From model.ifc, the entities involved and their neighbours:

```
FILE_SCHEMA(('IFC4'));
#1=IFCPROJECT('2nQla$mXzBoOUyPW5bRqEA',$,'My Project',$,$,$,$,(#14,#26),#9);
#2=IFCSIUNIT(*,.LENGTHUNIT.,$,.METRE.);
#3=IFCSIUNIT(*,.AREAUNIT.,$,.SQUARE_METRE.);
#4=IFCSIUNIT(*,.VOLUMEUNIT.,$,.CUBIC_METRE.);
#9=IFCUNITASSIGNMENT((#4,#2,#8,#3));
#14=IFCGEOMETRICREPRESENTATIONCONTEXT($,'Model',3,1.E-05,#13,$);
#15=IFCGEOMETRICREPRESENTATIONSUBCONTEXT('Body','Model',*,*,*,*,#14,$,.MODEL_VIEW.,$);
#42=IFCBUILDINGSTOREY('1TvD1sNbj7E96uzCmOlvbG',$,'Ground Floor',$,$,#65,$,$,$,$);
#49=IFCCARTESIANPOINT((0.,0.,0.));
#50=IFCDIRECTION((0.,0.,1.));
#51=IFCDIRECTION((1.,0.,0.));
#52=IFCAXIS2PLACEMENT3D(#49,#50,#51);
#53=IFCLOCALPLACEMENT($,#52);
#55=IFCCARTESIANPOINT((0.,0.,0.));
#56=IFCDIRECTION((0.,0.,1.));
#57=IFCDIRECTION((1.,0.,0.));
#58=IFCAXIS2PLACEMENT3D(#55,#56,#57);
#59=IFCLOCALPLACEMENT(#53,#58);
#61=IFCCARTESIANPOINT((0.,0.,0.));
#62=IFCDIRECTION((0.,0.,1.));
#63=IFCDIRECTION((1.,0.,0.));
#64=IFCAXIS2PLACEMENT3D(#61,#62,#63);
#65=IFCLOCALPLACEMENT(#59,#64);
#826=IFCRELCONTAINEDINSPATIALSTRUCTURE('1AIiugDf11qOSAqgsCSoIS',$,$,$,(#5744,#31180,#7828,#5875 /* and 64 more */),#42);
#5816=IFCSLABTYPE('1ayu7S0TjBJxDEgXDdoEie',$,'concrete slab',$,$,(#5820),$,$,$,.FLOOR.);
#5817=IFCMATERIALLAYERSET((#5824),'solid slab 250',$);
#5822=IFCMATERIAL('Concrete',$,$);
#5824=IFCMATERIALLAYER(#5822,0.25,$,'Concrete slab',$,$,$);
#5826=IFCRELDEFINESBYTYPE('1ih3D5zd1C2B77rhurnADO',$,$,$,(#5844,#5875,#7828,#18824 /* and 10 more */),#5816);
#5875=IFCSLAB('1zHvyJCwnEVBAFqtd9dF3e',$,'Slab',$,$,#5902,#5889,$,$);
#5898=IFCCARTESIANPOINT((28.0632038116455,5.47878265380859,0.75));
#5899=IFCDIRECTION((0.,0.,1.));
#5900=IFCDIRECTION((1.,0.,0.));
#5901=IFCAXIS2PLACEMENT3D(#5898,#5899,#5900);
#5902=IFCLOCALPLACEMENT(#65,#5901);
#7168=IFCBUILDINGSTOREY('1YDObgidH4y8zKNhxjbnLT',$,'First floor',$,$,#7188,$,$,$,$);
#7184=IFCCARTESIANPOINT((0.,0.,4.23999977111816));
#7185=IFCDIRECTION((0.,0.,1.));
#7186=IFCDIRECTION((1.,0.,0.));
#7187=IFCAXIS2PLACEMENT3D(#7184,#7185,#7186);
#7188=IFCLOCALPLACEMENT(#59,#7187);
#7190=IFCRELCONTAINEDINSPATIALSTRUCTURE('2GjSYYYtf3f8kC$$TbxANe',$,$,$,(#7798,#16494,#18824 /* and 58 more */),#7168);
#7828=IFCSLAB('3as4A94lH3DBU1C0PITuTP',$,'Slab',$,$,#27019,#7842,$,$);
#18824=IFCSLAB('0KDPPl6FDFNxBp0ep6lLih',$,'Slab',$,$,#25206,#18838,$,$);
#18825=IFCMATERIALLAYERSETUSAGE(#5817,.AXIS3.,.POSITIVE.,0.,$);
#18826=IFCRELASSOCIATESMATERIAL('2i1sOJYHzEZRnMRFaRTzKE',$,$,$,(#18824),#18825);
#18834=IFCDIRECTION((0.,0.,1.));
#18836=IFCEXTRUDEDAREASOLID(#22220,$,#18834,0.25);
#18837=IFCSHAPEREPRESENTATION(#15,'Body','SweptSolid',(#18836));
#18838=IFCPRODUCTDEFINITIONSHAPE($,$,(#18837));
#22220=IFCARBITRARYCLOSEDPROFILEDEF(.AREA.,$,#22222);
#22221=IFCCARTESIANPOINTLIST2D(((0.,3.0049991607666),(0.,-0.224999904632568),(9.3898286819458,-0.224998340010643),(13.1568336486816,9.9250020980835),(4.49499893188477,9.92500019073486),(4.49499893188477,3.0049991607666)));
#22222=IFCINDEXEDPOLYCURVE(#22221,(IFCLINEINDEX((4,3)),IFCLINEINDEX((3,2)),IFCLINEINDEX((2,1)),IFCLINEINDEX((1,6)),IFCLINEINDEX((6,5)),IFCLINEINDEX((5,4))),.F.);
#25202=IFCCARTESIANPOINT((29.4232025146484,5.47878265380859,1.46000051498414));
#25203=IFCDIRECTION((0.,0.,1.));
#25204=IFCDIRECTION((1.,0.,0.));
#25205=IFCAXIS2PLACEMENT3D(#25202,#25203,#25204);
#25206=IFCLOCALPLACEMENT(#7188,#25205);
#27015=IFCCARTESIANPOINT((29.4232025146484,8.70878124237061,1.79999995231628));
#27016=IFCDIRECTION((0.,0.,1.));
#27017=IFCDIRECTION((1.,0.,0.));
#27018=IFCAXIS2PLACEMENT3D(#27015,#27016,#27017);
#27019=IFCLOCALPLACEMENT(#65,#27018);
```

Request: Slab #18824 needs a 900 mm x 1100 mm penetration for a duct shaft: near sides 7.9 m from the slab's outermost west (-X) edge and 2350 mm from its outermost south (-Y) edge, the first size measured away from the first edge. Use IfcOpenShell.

```python
import numpy as np
import ifcopenshell
import ifcopenshell.api.feature
import ifcopenshell.api.geometry
import ifcopenshell.api.root
import ifcopenshell.geom
import ifcopenshell.util.placement
import ifcopenshell.util.representation
import ifcopenshell.util.shape
import ifcopenshell.util.unit

model = ifcopenshell.open("model.ifc")
unit_scale = ifcopenshell.util.unit.calculate_unit_scale(model)
settings = ifcopenshell.geom.settings()


def volume(element):
    """Net volume in cubic metres, openings subtracted."""
    shape = ifcopenshell.geom.create_shape(settings, element)
    return ifcopenshell.util.shape.get_volume(shape.geometry)


slab = model.by_guid("0KDPPl6FDFNxBp0ep6lLih")
before = volume(slab)

# Extent in the slab's own axes, in metres. The edges named are its -X and -Y sides.
slab_shape = ifcopenshell.geom.create_shape(settings, slab)
vertices = ifcopenshell.util.shape.get_vertices(slab_shape.geometry)
x_min, y_min, bottom = vertices.min(axis=0)
top = vertices[:, 2].max()

opening = ifcopenshell.api.root.create_entity(model, ifc_class="IfcOpeningElement", name="Duct shaft opening", predefined_type="OPENING")
context = ifcopenshell.util.representation.get_context(model, "Model", "Body", "MODEL_VIEW")
width, depth = 0.9, 1.1
outline = [(0.0, 0.0), (width, 0.0), (width, depth), (0.0, depth), (0.0, 0.0)]
# Overshoot both faces by 50 mm so the cut is clean.
shape = ifcopenshell.api.geometry.add_slab_representation(
    model, context=context, depth=top - bottom + 0.1, polyline=outline
)
ifcopenshell.api.geometry.assign_representation(model, product=opening, representation=shape)

matrix = ifcopenshell.util.placement.get_local_placement(slab.ObjectPlacement)
matrix[:, 3] = matrix @ np.append(np.array([x_min + 7.9, y_min + 2.35, bottom - 0.05]) / unit_scale, 1.0)
ifcopenshell.api.geometry.edit_object_placement(model, product=opening, matrix=matrix, is_si=False)
ifcopenshell.api.feature.add_feature(model, feature=opening, element=slab)

after = volume(slab)

print(f"slab volume {before:.3f} -> {after:.3f} m3")

model.write("model_v2.ifc")
```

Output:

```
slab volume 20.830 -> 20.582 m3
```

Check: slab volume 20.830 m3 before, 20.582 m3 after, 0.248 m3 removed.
